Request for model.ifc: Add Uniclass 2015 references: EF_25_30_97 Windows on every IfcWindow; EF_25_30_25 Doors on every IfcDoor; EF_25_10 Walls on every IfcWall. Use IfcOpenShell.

First a look at what the model holds.

```python
import ifcopenshell

model = ifcopenshell.open("model.ifc")
print(model.schema)
print("classifications:", [c.Name for c in model.by_type("IfcClassification")])
for ifc_class in ("IfcDoor", "IfcRoof", "IfcStair", "IfcWall", "IfcWindow"):
    print(ifc_class, len(model.by_type(ifc_class)))
```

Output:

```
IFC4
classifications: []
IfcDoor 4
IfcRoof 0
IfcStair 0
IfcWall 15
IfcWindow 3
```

```python
import ifcopenshell
import ifcopenshell.api.classification

model = ifcopenshell.open("model.ifc")

system = ifcopenshell.api.classification.add_classification(model, classification="Uniclass 2015")

codes = {
    "IfcWindow": ("EF_25_30_97", "Windows"),
    "IfcDoor": ("EF_25_30_25", "Doors"),
    "IfcWall": ("EF_25_10", "Walls"),
}
for ifc_class, (code, name) in codes.items():
    products = model.by_type(ifc_class)
    ifcopenshell.api.classification.add_reference(
        model, products=products, classification=system, identification=code, name=name
    )
    print(code, len(products))

model.write("model_edited.ifc")
```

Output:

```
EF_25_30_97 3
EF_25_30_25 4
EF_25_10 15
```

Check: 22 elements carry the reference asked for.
